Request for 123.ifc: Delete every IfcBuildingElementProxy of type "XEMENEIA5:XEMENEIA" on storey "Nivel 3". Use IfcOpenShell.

First a look at what the model holds.

```python
import ifcopenshell
import ifcopenshell.util.element

model = ifcopenshell.open("123.ifc")
print(model.schema)
storey = next(s for s in model.by_type("IfcBuildingStorey") if s.Name == "Nivel 3")
proxies = [e for e in ifcopenshell.util.element.get_decomposition(storey) if e.is_a("IfcBuildingElementProxy")]
seen = {}
for e in proxies:
    element_type = ifcopenshell.util.element.get_type(e)
    name = element_type.Name if element_type not in (None, e) else None
    seen[name] = seen.get(name, 0) + 1
for name, count in sorted(seen.items(), key=str):
    print(count, "x", name)
```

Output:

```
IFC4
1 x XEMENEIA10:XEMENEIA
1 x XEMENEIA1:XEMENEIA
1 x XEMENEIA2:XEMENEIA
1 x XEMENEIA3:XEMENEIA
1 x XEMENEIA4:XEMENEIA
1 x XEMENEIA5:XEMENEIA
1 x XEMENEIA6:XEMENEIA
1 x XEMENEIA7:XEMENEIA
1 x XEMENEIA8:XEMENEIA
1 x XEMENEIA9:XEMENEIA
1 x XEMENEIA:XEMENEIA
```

```python
import ifcopenshell
import ifcopenshell.api.root
import ifcopenshell.util.element

model = ifcopenshell.open("123.ifc")

storey = next(s for s in model.by_type("IfcBuildingStorey") if s.Name == "Nivel 3")
proxies = [e for e in ifcopenshell.util.element.get_decomposition(storey) if e.is_a("IfcBuildingElementProxy")]
targets = [e for e in proxies if (t := ifcopenshell.util.element.get_type(e)) not in (None, e) and t.Name == "XEMENEIA5:XEMENEIA"]

for e in targets:
    ifcopenshell.api.root.remove_product(model, product=e)
print(len(targets), "removed")

model.write("123-out.ifc")
```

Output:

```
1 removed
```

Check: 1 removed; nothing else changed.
